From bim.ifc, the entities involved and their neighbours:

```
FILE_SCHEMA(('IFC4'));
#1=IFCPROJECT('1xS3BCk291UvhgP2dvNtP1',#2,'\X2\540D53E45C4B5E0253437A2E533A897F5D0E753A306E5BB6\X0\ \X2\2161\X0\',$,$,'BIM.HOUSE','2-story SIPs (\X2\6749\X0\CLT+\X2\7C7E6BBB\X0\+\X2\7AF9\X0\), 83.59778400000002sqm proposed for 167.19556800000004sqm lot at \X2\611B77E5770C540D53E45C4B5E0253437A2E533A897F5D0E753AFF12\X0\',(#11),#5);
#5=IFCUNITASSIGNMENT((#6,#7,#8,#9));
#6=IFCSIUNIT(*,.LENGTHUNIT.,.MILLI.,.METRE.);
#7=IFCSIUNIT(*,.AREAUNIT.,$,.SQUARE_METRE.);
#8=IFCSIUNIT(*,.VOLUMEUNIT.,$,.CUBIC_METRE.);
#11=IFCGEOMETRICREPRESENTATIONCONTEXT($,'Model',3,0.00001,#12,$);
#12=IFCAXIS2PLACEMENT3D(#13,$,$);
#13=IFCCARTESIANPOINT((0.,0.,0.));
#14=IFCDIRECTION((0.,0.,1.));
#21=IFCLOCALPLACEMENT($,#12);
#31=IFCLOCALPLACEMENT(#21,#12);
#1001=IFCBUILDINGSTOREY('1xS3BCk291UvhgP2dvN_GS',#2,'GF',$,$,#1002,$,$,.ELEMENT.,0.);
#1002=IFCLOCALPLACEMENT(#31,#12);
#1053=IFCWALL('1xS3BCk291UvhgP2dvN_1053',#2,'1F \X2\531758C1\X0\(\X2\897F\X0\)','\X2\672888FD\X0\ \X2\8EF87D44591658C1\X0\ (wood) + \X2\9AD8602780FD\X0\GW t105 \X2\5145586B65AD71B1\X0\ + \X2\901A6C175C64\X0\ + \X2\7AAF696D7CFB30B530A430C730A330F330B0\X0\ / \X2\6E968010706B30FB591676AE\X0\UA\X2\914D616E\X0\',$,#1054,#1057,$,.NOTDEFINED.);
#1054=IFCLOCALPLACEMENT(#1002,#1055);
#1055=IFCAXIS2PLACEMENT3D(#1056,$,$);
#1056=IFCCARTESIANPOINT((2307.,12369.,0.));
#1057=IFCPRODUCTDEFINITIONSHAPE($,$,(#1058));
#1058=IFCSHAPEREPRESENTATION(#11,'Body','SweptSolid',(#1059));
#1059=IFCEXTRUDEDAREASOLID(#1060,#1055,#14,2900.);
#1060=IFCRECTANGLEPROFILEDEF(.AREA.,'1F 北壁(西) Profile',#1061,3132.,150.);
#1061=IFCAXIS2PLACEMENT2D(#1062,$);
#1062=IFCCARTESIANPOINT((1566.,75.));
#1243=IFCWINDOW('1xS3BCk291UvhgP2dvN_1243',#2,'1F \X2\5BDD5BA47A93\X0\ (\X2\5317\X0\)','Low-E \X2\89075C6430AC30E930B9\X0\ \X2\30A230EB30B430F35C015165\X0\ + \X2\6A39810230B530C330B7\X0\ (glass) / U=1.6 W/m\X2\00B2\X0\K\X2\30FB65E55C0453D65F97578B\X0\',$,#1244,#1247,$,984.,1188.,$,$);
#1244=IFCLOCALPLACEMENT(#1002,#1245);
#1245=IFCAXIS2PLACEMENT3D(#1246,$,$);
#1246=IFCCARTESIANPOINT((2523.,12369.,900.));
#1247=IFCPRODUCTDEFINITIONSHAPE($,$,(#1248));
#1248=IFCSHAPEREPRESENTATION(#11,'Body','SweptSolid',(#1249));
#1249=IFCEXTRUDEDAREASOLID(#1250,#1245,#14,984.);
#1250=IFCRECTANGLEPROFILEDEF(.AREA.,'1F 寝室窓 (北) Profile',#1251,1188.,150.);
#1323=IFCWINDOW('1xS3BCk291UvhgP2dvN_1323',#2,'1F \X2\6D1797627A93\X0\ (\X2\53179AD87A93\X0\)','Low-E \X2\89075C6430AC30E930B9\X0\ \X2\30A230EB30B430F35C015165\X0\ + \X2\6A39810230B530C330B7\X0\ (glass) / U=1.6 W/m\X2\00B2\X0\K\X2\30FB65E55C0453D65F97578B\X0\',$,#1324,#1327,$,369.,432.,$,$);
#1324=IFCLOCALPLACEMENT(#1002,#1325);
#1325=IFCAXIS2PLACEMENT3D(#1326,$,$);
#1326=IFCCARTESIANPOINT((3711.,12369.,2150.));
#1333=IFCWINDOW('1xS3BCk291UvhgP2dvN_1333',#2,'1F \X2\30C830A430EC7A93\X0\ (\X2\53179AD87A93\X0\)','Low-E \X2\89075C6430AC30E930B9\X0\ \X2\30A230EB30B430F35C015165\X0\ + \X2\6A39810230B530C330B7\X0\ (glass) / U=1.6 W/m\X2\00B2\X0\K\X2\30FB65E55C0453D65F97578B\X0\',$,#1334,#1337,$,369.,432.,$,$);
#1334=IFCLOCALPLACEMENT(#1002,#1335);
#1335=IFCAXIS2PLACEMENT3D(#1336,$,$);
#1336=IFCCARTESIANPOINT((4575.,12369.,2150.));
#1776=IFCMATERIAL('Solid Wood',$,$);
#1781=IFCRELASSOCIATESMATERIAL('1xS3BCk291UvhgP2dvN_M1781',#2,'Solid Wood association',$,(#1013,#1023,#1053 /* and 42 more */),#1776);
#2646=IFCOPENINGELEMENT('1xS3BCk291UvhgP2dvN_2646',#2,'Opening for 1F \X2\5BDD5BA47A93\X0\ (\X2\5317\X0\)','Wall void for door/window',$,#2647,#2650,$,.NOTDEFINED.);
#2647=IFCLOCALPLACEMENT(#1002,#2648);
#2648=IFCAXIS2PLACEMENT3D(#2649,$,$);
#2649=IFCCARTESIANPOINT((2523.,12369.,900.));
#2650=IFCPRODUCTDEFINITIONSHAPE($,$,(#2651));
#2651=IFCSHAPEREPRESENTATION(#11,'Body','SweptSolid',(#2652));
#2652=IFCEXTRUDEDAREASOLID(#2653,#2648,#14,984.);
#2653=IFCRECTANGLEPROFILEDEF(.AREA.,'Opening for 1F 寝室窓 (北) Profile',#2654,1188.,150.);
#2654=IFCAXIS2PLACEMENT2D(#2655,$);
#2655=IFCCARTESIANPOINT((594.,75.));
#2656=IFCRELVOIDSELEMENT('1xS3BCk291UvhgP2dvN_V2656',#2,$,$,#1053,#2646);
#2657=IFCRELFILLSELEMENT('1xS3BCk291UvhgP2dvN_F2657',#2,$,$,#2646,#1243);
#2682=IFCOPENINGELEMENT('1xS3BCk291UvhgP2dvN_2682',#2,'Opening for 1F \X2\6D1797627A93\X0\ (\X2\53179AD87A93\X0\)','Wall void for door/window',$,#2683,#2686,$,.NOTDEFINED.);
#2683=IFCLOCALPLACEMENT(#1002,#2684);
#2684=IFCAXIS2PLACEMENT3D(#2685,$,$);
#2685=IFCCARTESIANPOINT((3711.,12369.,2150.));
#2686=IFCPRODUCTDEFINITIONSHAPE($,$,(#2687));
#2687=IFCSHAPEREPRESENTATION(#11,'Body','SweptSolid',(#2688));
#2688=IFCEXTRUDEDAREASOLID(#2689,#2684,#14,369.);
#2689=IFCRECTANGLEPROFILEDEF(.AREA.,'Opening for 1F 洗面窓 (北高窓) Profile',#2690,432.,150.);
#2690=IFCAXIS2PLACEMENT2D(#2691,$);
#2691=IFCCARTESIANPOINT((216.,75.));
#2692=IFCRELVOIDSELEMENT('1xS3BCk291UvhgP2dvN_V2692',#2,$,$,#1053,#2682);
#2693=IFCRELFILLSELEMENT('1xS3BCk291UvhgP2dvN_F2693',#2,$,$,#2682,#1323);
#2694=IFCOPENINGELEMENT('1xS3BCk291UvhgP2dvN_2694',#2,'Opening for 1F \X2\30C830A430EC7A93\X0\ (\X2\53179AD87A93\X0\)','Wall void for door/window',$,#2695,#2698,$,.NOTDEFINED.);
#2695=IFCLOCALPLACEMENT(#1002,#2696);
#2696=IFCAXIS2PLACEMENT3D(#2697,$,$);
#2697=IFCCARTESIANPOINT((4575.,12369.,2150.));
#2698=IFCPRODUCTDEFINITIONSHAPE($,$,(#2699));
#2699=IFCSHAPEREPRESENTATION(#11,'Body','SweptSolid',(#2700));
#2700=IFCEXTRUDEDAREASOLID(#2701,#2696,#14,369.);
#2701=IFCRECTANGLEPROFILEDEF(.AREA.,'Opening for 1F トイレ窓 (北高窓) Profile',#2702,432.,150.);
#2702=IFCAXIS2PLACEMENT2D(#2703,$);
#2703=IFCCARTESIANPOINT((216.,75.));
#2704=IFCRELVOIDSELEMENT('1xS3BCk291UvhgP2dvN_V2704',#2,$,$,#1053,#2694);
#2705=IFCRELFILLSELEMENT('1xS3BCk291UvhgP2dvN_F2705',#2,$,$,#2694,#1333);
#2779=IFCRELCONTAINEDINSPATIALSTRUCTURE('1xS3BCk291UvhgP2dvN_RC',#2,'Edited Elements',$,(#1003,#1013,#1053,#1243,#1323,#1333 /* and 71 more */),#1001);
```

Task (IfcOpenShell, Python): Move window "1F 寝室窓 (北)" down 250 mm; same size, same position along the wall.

```python
import numpy as np
import ifcopenshell
import ifcopenshell.api.geometry
import ifcopenshell.util.placement
import ifcopenshell.util.unit

model = ifcopenshell.open("bim.ifc")
unit_scale = ifcopenshell.util.unit.calculate_unit_scale(model)

window = model.by_guid("1xS3BCk291UvhgP2dvN_1243")
opening = window.FillsVoids[0].RelatingOpeningElement
dz = -0.25 / unit_scale

shift = np.array([0.0, 0.0, dz])
# The window is not placed relative to its opening, so move both.
for product in (opening, window):
    matrix = ifcopenshell.util.placement.get_local_placement(product.ObjectPlacement)
    matrix[:3, 3] += shift
    ifcopenshell.api.geometry.edit_object_placement(model, product=product, matrix=matrix, is_si=False)

print(f"moved by {dz * unit_scale:+.3f} m")

model.write("bim-out.ifc")
```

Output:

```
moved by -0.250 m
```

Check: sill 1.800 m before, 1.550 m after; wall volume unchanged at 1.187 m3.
